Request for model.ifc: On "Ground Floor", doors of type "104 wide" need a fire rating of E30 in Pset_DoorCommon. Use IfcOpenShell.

First a look at what the model holds.

```python
import ifcopenshell
import ifcopenshell.util.element

model = ifcopenshell.open("model.ifc")
print(model.schema)
storey = next(s for s in model.by_type("IfcBuildingStorey") if s.Name == "Ground Floor")
doors = [e for e in ifcopenshell.util.element.get_decomposition(storey) if e.is_a("IfcDoor")]
seen = {}
for e in doors:
    element_type = ifcopenshell.util.element.get_type(e)
    key = (element_type.Name if element_type != e and element_type else None, ifcopenshell.util.element.get_pset(e, "Pset_DoorCommon", "FireRating"))
    seen[key] = seen.get(key, 0) + 1
for (name, value), count in sorted(seen.items(), key=str):
    print(count, "x", name, "|", value)
```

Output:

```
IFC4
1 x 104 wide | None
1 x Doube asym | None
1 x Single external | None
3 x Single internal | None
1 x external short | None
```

```python
import ifcopenshell
import ifcopenshell.api.pset
import ifcopenshell.util.element

model = ifcopenshell.open("model.ifc")

storey = next(s for s in model.by_type("IfcBuildingStorey") if s.Name == "Ground Floor")
doors = [e for e in ifcopenshell.util.element.get_decomposition(storey) if e.is_a("IfcDoor")]

count = 0
for e in doors:
    element_type = ifcopenshell.util.element.get_type(e)
    if element_type in (None, e) or element_type.Name != "104 wide":
        continue
    # add_pset returns the element's existing set when there is one.
    pset = ifcopenshell.api.pset.add_pset(model, product=e, name="Pset_DoorCommon")
    ifcopenshell.api.pset.edit_pset(model, pset=pset, properties={"FireRating": "E30"})
    count += 1

print(count, "doors updated")

model.write("model-out.ifc")
```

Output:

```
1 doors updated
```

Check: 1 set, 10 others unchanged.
